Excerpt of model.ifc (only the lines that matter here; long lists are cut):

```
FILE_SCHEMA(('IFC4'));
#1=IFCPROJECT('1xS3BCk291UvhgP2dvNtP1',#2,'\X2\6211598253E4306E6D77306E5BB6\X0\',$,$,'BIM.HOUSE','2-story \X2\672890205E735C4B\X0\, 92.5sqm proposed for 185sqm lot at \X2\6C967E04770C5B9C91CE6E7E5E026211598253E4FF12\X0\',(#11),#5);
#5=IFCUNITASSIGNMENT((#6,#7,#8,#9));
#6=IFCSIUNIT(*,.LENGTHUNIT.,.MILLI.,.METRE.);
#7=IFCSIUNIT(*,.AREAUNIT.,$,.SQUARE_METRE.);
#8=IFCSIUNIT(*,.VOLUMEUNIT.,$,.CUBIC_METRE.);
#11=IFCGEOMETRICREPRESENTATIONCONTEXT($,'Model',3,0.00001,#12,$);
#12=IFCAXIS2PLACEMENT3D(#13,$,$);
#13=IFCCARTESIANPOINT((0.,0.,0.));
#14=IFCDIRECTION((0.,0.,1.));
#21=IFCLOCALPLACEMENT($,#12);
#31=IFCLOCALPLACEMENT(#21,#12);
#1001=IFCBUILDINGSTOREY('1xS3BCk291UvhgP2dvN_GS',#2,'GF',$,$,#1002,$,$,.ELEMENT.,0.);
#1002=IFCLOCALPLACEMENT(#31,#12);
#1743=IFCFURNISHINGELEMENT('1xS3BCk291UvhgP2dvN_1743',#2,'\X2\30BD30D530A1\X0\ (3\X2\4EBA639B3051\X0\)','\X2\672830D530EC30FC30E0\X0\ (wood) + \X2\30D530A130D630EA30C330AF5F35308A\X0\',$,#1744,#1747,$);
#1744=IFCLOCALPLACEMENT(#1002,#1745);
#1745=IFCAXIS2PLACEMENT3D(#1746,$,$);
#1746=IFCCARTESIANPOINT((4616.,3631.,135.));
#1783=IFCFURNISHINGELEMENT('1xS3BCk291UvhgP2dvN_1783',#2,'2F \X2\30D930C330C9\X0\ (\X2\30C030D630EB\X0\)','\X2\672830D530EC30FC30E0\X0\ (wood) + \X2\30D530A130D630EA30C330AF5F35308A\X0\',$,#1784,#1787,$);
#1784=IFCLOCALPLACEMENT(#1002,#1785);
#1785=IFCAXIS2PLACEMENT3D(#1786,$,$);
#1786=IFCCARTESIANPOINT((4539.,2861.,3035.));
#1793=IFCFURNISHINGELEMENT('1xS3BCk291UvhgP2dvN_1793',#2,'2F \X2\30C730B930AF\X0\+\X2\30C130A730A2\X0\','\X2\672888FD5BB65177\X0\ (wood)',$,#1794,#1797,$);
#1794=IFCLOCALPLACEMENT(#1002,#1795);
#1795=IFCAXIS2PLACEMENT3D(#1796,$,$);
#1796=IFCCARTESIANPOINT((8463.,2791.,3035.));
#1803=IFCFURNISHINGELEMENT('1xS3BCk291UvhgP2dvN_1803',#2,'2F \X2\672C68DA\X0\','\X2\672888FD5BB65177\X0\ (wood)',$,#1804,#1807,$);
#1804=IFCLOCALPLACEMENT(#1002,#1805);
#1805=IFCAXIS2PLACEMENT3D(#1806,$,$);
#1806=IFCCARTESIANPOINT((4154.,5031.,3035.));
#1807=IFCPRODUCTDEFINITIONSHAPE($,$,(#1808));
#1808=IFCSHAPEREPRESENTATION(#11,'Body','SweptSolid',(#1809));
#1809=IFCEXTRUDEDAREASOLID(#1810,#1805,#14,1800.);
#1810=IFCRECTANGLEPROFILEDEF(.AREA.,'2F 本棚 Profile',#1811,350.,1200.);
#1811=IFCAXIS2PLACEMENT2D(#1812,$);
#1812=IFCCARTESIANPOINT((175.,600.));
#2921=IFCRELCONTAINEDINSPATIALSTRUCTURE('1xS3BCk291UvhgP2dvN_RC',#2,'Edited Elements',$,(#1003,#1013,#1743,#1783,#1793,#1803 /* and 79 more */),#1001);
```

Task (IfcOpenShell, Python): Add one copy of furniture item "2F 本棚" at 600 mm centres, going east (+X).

```python
import numpy as np
import ifcopenshell
import ifcopenshell.api.geometry
import ifcopenshell.api.root
import ifcopenshell.util.element
import ifcopenshell.util.placement
import ifcopenshell.util.unit

model = ifcopenshell.open("model.ifc")
unit_scale = ifcopenshell.util.unit.calculate_unit_scale(model)


def reuse_history(source, copy):
    """copy_class also copies each property set's owner history, people and application; keep the originals."""
    for rel in copy.IsDefinedBy:
        if rel.is_a("IfcRelDefinesByProperties") and (history := rel.RelatingPropertyDefinition.OwnerHistory):
            rel.RelatingPropertyDefinition.OwnerHistory = source.OwnerHistory
            ifcopenshell.util.element.remove_deep2(model, history)


source = model.by_id(1803)
base = ifcopenshell.util.placement.get_local_placement(source.ObjectPlacement)
step = np.array([1.0, 0.0, 0.0]) * 0.6 / unit_scale

for i in range(1, 2):
    copy = ifcopenshell.api.root.copy_class(model, product=source)
    copy.Representation = ifcopenshell.util.element.copy_deep(
        model, source.Representation, exclude=["IfcGeometricRepresentationContext", "IfcRepresentationMap"]
    )
    reuse_history(source, copy)
    matrix = base.copy()
    matrix[:3, 3] += i * step
    print("added at", matrix[:3, 3].round(3) + 0.0)
    ifcopenshell.api.geometry.edit_object_placement(model, product=copy, matrix=matrix, is_si=False)

model.write("model_edited.ifc")
```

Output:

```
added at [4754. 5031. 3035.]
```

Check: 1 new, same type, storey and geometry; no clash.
